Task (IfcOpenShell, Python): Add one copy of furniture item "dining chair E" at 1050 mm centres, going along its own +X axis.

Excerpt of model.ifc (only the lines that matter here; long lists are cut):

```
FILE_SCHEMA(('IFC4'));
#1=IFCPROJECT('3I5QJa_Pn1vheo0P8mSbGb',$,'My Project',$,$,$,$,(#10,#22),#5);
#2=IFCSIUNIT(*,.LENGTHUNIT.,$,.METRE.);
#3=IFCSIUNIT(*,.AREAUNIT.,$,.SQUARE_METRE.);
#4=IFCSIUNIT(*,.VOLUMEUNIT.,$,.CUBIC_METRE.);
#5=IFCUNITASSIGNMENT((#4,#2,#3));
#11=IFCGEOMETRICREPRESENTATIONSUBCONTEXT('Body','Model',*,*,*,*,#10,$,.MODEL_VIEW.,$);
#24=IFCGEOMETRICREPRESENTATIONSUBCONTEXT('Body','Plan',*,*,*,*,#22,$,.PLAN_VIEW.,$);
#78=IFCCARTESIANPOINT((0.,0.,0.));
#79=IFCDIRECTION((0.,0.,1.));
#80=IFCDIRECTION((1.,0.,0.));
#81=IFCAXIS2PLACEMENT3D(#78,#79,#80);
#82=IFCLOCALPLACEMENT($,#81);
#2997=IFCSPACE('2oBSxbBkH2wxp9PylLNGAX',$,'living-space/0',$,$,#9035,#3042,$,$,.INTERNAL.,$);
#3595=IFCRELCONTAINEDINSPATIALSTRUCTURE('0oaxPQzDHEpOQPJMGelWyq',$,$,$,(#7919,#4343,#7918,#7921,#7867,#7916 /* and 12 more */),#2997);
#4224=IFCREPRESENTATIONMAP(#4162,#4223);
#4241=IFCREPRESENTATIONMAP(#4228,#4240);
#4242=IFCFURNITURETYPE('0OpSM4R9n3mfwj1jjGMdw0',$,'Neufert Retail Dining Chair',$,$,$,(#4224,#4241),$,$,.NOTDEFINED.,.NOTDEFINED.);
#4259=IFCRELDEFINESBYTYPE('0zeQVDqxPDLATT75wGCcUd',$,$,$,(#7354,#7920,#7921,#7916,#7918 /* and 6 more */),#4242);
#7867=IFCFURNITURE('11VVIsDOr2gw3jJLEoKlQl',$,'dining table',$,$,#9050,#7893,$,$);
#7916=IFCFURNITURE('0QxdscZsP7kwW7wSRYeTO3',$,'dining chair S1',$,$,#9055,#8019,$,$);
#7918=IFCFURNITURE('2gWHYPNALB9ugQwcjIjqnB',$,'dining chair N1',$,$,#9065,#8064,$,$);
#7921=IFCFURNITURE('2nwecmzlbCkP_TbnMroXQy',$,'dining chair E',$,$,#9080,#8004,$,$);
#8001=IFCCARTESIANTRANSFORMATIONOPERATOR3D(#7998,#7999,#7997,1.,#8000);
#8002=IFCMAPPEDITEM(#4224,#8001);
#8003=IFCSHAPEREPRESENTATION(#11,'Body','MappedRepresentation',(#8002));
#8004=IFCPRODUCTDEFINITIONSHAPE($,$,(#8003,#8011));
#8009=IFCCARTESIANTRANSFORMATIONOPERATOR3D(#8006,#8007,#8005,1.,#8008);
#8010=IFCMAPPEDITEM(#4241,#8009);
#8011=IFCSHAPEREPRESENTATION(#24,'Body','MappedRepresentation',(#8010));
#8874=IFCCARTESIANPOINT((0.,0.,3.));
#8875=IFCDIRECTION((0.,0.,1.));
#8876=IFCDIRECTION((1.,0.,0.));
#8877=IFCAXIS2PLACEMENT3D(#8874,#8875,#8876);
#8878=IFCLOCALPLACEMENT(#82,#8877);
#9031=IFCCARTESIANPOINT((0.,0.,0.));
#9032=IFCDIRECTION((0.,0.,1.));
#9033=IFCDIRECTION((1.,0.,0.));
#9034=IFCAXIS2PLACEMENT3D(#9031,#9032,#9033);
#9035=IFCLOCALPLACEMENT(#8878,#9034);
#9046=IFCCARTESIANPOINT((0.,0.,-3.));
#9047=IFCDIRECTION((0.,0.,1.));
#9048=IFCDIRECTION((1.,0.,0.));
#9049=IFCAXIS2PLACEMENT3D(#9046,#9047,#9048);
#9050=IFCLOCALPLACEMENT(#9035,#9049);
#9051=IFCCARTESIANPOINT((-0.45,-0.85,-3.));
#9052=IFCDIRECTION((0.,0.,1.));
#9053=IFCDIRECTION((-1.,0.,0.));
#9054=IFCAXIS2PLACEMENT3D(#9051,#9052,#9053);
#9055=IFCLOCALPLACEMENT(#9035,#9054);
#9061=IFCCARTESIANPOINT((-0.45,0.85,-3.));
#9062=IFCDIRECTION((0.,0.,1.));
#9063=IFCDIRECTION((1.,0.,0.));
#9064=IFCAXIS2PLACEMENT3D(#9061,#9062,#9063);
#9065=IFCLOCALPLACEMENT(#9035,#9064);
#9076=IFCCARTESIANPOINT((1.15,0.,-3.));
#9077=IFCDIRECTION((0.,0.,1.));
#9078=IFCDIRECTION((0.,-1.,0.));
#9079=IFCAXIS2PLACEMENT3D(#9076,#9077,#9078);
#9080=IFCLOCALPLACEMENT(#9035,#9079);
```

```python
import ifcopenshell
import ifcopenshell.api.geometry
import ifcopenshell.api.root
import ifcopenshell.util.element
import ifcopenshell.util.placement
import ifcopenshell.util.unit

model = ifcopenshell.open("model.ifc")
unit_scale = ifcopenshell.util.unit.calculate_unit_scale(model)

source = model.by_guid("2nwecmzlbCkP_TbnMroXQy")
base = ifcopenshell.util.placement.get_local_placement(source.ObjectPlacement)
step = base[:3, 0] * 1.05 / unit_scale

for i in range(1, 2):
    copy = ifcopenshell.api.root.copy_class(model, product=source)
    copy.Representation = ifcopenshell.util.element.copy_deep(
        model, source.Representation, exclude=["IfcGeometricRepresentationContext", "IfcRepresentationMap"]
    )
    matrix = base.copy()
    matrix[:3, 3] += i * step
    print("added at", matrix[:3, 3].round(3) + 0.0)
    ifcopenshell.api.geometry.edit_object_placement(model, product=copy, matrix=matrix, is_si=False)

model.write("model-out.ifc")
```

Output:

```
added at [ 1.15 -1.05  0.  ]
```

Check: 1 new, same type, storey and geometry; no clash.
